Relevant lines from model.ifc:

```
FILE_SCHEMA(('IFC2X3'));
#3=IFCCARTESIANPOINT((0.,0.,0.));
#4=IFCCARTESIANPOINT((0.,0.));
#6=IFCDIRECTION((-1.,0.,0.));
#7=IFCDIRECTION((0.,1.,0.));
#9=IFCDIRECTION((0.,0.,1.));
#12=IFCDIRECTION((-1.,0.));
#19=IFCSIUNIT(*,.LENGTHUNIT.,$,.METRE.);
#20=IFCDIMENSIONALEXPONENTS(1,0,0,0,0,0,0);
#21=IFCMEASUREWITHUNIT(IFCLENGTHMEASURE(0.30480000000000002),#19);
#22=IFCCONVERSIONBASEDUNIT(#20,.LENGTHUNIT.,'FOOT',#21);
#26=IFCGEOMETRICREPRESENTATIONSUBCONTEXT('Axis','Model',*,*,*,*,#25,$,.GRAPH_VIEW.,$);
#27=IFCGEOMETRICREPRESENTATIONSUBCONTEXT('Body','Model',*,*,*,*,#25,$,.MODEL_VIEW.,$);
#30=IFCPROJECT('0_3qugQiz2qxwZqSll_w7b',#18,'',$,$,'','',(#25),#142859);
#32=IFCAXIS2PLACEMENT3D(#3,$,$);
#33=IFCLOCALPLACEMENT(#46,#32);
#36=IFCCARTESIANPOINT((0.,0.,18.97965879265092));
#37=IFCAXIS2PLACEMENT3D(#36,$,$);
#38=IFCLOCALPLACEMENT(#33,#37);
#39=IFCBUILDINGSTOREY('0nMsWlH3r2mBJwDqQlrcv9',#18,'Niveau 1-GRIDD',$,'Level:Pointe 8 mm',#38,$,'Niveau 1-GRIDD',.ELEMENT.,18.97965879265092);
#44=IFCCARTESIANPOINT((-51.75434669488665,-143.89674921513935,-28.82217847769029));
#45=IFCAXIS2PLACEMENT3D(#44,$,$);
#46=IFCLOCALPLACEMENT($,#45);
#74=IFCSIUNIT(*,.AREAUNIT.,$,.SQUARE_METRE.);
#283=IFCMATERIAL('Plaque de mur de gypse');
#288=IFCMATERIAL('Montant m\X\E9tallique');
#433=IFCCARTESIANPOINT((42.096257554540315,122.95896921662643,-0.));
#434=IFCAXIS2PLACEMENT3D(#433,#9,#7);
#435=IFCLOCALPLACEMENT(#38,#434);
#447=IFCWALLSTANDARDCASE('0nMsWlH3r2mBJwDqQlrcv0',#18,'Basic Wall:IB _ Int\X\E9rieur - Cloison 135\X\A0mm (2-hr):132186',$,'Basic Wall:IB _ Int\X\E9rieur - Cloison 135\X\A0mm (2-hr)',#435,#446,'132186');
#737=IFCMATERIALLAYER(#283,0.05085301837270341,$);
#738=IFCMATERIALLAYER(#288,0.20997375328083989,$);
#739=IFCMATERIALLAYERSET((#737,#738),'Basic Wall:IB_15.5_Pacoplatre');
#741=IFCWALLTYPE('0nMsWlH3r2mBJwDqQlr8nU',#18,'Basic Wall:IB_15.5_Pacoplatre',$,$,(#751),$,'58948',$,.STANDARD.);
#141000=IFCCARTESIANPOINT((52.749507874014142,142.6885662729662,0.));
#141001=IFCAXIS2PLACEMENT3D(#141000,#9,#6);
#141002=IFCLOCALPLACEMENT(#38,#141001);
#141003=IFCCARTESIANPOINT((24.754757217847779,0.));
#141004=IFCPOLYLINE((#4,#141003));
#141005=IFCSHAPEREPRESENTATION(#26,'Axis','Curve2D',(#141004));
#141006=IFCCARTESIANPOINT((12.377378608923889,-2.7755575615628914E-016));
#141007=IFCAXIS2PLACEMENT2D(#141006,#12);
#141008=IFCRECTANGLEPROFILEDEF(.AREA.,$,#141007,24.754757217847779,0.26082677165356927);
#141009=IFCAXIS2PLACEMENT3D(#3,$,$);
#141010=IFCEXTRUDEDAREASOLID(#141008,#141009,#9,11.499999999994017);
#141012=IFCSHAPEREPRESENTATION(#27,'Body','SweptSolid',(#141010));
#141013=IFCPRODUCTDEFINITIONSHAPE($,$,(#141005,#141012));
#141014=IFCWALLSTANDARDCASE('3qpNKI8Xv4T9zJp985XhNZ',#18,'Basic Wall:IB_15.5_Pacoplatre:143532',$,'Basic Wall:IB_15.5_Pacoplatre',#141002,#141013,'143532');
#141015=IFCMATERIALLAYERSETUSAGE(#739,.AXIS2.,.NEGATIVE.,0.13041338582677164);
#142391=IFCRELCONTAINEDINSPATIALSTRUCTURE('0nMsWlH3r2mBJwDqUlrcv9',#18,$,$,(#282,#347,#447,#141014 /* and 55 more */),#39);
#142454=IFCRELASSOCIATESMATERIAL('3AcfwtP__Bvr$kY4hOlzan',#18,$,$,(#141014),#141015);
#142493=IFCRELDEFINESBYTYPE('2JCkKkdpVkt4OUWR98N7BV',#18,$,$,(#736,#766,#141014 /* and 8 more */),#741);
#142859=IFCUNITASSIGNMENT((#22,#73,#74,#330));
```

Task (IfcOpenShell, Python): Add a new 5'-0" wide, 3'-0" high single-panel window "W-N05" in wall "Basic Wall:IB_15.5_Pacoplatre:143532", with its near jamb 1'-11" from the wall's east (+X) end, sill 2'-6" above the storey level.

```python
import numpy as np
import ifcopenshell
import ifcopenshell.api.feature
import ifcopenshell.api.geometry
import ifcopenshell.api.root
import ifcopenshell.api.spatial
import ifcopenshell.api.type
import ifcopenshell.geom
import ifcopenshell.util.element
import ifcopenshell.util.placement
import ifcopenshell.util.representation
import ifcopenshell.util.shape
import ifcopenshell.util.unit

model = ifcopenshell.open("model.ifc")
unit_scale = ifcopenshell.util.unit.calculate_unit_scale(model)
settings = ifcopenshell.geom.settings()


def volume(element):
    """Net volume in cubic metres, openings subtracted."""
    shape = ifcopenshell.geom.create_shape(settings, element)
    return ifcopenshell.util.shape.get_volume(shape.geometry)


wall = model.by_guid("3qpNKI8Xv4T9zJp985XhNZ")
storey = ifcopenshell.util.element.get_container(wall, ifc_class="IfcBuildingStorey")
context = ifcopenshell.util.representation.get_context(model, "Model", "Body", "MODEL_VIEW")
before = volume(wall)

width, height, from_end, sill = 1.524, 0.9144, 0.5842, 0.762  # metres

# The wall runs along its own X axis, and the end named is its -X end.
wall_shape = ifcopenshell.geom.create_shape(settings, wall)
x, y, z = ifcopenshell.util.shape.get_vertices(wall_shape.geometry).T
start = x.min() + from_end
face, thickness = float(y.min()), float(y.max() - y.min())
wall_matrix = ifcopenshell.util.placement.get_local_placement(wall.ObjectPlacement)
level = ifcopenshell.util.placement.get_local_placement(storey.ObjectPlacement)[2, 3]


def in_wall(x, y):
    """Placement at x, y metres in the wall's axes, at sill height."""
    matrix = wall_matrix.copy()
    matrix[:, 3] = wall_matrix @ np.array([x / unit_scale, y / unit_scale, 0.0, 1.0])
    matrix[2, 3] = level + sill / unit_scale
    return matrix


# Opening: a box that overshoots both wall faces by 50 mm.
opening = ifcopenshell.api.root.create_entity(model, ifc_class="IfcOpeningElement")
box = ifcopenshell.api.geometry.add_wall_representation(
    model, context=context, length=width, height=height, thickness=thickness + 0.1
)
ifcopenshell.api.geometry.assign_representation(model, product=opening, representation=box)
ifcopenshell.api.geometry.edit_object_placement(model, product=opening, matrix=in_wall(start, face - 0.05), is_si=False)
ifcopenshell.api.feature.add_feature(model, feature=opening, element=wall)

window = ifcopenshell.api.root.create_entity(model, ifc_class="IfcWindow", name="W-N05")
window.OverallWidth, window.OverallHeight = width / unit_scale, height / unit_scale
body = ifcopenshell.api.geometry.add_window_representation(
    model,
    context=context,
    overall_width=window.OverallWidth,
    overall_height=window.OverallHeight,
    partition_type="SINGLE_PANEL",
)
ifcopenshell.api.geometry.assign_representation(model, product=window, representation=body)
ifcopenshell.api.spatial.assign_container(model, products=[window], relating_structure=storey)
fills = ifcopenshell.api.feature.add_filling(model, opening=opening, element=window)
fills.OwnerHistory = window.OwnerHistory  # required in IFC2X3

# IFC2X3 keeps the operation on the window style.
style = ifcopenshell.api.root.create_entity(model, ifc_class="IfcWindowStyle", name="W-N05")
style.OperationType, style.ConstructionType = "SINGLE_PANEL", "NOTDEFINED"
style.ParameterTakesPrecedence = style.Sizeable = False
ifcopenshell.api.type.assign_type(model, related_objects=[window], relating_type=style)

# Centre the window in the wall's thickness.
ifcopenshell.api.geometry.edit_object_placement(model, product=window, matrix=in_wall(start, face), is_si=False)
window_shape = ifcopenshell.geom.create_shape(settings, window)
depth = ifcopenshell.util.shape.get_vertices(window_shape.geometry)[:, 1]
offset = face + thickness / 2 - (depth.min() + depth.max()) / 2
ifcopenshell.api.geometry.edit_object_placement(model, product=window, matrix=in_wall(start, offset), is_si=False)

after = volume(wall)

print(f"wall volume {before:.3f} -> {after:.3f} m3")

model.write("model_edited.ifc")
```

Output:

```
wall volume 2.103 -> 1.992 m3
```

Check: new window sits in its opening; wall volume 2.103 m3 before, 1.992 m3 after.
